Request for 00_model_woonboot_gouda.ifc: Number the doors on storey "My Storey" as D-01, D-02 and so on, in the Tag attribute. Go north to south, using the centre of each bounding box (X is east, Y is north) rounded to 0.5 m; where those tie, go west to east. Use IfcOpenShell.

First a look at what the model holds.

```python
import ifcopenshell
import ifcopenshell.util.element
import ifcopenshell.util.placement

model = ifcopenshell.open("00_model_woonboot_gouda.ifc")
print(model.schema)
storey = next(s for s in model.by_type("IfcBuildingStorey") if s.Name == "My Storey")
doors = [e for e in ifcopenshell.util.element.get_decomposition(storey) if e.is_a("IfcDoor")]
for e in sorted(doors, key=lambda e: e.id()):
    origin = ifcopenshell.util.placement.get_local_placement(e.ObjectPlacement)[:3, 3]
    print(e.id(), e.Tag, e.Name, origin.round(2) + 0.0, sep=" | ")
```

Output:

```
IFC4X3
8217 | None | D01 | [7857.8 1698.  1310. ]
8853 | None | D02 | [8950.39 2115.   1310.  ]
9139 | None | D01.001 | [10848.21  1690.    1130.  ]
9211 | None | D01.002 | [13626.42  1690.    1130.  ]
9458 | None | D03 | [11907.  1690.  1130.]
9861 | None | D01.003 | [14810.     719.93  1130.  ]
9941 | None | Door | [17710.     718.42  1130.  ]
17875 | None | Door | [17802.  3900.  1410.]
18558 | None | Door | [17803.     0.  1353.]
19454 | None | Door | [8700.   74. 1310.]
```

```python
import ifcopenshell
import ifcopenshell.geom
import ifcopenshell.util.element
import ifcopenshell.util.shape

model = ifcopenshell.open("00_model_woonboot_gouda.ifc")
settings = ifcopenshell.geom.settings()
settings.set("use-world-coords", True)


def centre(element):
    shape = ifcopenshell.geom.create_shape(settings, element)
    return ifcopenshell.util.shape.get_bbox_centroid(shape.geometry)


storey = next(s for s in model.by_type("IfcBuildingStorey") if s.Name == "My Storey")
doors = [e for e in ifcopenshell.util.element.get_decomposition(storey) if e.is_a("IfcDoor")]

# Insertion points can sit at a corner or the storey origin, so sort by the geometry (in metres).
centres = {e: centre(e) for e in doors}
doors.sort(key=lambda e: (-round(centres[e][1] / 0.5), centres[e][0]))

for i, e in enumerate(doors, start=1):
    number = f"D-{i:02d}"
    e.Tag = number
    print(e.id(), number)

model.write("00_model_woonboot_gouda_rev.ifc")
```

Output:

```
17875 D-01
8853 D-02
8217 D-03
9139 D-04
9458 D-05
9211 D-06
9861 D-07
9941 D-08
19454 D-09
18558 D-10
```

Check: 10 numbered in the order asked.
